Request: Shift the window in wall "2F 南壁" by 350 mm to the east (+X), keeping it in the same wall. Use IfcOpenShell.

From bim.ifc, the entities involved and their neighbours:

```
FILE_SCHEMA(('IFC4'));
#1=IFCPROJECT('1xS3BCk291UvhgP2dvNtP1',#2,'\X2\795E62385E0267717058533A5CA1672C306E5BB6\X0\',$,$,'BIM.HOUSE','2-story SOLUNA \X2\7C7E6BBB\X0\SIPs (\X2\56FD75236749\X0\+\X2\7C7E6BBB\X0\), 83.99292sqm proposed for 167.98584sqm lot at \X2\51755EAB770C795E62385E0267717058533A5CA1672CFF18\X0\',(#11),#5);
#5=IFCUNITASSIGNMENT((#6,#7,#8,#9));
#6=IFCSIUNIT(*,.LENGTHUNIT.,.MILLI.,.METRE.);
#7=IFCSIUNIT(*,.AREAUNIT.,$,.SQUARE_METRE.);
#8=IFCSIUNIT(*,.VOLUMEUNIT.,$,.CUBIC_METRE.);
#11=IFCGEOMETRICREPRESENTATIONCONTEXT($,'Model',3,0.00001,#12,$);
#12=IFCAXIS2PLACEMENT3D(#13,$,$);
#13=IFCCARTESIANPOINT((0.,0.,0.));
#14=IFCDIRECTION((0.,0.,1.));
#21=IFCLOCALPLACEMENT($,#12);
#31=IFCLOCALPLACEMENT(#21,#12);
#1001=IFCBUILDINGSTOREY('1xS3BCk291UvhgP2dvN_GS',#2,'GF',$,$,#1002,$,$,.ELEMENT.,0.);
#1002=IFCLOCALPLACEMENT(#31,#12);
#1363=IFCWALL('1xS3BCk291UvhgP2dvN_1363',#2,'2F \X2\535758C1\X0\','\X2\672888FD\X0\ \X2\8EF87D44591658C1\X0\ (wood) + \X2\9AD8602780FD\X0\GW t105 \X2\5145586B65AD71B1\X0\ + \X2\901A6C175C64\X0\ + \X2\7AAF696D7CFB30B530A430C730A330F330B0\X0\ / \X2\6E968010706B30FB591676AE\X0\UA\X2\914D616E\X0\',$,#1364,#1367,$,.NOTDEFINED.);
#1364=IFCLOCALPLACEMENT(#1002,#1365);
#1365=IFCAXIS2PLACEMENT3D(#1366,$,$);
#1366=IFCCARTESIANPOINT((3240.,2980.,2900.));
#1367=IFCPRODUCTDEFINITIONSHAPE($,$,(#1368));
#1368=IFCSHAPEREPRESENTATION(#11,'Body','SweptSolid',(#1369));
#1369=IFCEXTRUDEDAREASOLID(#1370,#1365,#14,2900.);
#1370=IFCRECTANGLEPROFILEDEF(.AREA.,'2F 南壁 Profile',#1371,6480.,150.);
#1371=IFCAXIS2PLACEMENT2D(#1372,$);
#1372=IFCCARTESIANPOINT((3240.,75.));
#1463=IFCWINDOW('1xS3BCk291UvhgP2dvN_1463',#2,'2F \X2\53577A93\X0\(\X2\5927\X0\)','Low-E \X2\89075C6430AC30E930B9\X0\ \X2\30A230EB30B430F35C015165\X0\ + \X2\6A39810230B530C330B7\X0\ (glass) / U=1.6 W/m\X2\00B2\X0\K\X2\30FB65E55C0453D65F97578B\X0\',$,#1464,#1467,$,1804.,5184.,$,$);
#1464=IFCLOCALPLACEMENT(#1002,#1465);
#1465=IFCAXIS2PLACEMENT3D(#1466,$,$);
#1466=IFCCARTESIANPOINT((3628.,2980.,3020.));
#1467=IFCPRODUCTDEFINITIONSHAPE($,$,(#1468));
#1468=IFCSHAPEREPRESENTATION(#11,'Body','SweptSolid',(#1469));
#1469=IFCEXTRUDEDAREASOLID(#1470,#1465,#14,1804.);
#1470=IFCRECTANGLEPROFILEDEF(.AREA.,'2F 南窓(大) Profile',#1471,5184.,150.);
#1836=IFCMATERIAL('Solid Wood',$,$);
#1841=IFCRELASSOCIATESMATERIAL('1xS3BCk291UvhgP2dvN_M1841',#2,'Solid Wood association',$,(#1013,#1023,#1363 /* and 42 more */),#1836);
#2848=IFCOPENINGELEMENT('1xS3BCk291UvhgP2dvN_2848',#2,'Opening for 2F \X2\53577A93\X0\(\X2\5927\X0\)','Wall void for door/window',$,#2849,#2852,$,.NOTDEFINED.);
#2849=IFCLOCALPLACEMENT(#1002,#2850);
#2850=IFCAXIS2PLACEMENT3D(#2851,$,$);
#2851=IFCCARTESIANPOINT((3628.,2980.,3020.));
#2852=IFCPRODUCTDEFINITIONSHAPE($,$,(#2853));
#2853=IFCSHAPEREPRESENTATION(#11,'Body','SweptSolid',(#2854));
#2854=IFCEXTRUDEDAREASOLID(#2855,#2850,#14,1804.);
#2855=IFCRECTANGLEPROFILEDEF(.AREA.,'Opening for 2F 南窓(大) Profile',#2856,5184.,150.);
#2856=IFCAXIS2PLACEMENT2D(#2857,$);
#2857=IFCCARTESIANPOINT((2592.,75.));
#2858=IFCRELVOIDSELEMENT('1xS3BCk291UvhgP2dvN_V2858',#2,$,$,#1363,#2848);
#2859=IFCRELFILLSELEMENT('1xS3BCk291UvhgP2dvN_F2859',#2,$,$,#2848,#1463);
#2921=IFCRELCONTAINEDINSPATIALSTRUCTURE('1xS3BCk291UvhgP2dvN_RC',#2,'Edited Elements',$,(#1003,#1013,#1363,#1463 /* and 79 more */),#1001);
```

```python
import ifcopenshell
import ifcopenshell.api.geometry
import ifcopenshell.util.placement
import ifcopenshell.util.unit

model = ifcopenshell.open("bim.ifc")
unit_scale = ifcopenshell.util.unit.calculate_unit_scale(model)

window = model.by_guid("1xS3BCk291UvhgP2dvN_1463")
opening = window.FillsVoids[0].RelatingOpeningElement
wall = opening.VoidsElements[0].RelatingBuildingElement

wall_matrix = ifcopenshell.util.placement.get_local_placement(wall.ObjectPlacement)
shift = wall_matrix[:3, 0] * 0.35 / unit_scale
before = ifcopenshell.util.placement.get_local_placement(window.ObjectPlacement)[:3, 3].copy()

# The window is not placed relative to its opening, so move both.
for product in (opening, window):
    matrix = ifcopenshell.util.placement.get_local_placement(product.ObjectPlacement)
    matrix[:3, 3] += shift
    ifcopenshell.api.geometry.edit_object_placement(model, product=product, matrix=matrix, is_si=False)

after = ifcopenshell.util.placement.get_local_placement(window.ObjectPlacement)[:3, 3]
print("window moved by", (after - before).round(3) + 0.0)

model.write("bim_edited.ifc")
```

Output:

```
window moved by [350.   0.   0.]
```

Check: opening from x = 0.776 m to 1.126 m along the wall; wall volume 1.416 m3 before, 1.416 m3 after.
